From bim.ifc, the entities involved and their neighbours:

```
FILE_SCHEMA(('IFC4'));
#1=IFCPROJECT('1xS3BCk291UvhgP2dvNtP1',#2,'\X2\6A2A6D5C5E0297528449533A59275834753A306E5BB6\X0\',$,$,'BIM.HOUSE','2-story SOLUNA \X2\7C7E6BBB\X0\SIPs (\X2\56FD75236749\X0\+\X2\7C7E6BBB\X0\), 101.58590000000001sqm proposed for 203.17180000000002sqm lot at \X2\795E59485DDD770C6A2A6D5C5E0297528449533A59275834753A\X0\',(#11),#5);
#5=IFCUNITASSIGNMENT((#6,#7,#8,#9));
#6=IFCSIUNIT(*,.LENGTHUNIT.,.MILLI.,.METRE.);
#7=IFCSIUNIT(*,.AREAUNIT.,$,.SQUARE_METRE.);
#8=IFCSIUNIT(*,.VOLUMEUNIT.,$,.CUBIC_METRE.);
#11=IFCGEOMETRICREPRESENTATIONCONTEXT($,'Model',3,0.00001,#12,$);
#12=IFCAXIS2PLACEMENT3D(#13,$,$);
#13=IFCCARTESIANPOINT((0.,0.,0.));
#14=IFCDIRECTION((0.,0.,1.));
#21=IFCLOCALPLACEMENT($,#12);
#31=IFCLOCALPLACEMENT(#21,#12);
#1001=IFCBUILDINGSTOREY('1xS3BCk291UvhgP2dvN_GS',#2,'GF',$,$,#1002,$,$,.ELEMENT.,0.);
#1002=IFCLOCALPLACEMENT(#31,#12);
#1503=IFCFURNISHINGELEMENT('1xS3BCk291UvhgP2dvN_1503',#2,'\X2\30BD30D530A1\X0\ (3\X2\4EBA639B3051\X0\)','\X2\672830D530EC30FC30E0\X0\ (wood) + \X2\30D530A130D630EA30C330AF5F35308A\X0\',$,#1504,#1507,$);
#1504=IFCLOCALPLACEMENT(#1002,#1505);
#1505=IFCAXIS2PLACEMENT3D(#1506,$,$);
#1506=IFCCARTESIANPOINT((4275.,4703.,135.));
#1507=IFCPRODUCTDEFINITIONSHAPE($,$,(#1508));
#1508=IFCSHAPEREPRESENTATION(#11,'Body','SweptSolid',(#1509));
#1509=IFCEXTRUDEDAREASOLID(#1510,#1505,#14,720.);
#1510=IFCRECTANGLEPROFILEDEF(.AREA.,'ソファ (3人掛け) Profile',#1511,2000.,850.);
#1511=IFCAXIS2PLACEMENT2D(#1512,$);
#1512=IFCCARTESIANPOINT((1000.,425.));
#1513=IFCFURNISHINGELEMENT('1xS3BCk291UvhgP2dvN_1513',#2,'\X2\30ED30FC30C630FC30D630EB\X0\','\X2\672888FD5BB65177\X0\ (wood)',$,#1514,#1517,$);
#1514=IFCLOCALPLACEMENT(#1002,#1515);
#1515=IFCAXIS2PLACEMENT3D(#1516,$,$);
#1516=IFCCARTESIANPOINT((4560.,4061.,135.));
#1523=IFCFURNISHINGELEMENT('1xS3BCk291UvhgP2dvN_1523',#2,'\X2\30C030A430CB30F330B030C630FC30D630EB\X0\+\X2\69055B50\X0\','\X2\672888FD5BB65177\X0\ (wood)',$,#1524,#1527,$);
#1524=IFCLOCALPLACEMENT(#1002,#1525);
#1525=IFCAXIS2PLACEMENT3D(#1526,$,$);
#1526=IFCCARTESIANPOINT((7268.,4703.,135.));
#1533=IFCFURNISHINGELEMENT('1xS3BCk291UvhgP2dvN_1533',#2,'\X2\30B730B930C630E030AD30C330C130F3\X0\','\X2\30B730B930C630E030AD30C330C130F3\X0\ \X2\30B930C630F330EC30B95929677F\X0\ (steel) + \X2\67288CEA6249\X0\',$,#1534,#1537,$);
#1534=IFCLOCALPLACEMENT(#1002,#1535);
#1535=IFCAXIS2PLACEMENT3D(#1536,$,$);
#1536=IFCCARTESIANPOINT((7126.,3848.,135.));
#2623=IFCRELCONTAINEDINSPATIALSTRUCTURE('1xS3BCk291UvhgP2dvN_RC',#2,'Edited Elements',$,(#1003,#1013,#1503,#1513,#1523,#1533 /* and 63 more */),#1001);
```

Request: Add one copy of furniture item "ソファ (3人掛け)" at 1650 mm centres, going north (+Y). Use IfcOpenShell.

```python
import numpy as np
import ifcopenshell
import ifcopenshell.api.geometry
import ifcopenshell.api.root
import ifcopenshell.util.element
import ifcopenshell.util.placement

model = ifcopenshell.open("bim.ifc")


def reuse_history(source, copy):
    """copy_class also copies each property set's owner history, people and application; keep the originals."""
    for rel in copy.IsDefinedBy:
        if rel.is_a("IfcRelDefinesByProperties") and (history := rel.RelatingPropertyDefinition.OwnerHistory):
            rel.RelatingPropertyDefinition.OwnerHistory = source.OwnerHistory
            ifcopenshell.util.element.remove_deep2(model, history)


source = model.by_guid("1xS3BCk291UvhgP2dvN_1503")
base = ifcopenshell.util.placement.get_local_placement(source.ObjectPlacement)
step = np.array([0.0, 1.0, 0.0]) * 1650.0

for i in range(1, 2):
    copy = ifcopenshell.api.root.copy_class(model, product=source)
    copy.Representation = ifcopenshell.util.element.copy_deep(
        model, source.Representation, exclude=["IfcGeometricRepresentationContext", "IfcRepresentationMap"]
    )
    reuse_history(source, copy)
    matrix = base.copy()
    matrix[:3, 3] += i * step
    print("added at", matrix[:3, 3].round(3) + 0.0)
    ifcopenshell.api.geometry.edit_object_placement(model, product=copy, matrix=matrix, is_si=False)

model.write("bim-out.ifc")
```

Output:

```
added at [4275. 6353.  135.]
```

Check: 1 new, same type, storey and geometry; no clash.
